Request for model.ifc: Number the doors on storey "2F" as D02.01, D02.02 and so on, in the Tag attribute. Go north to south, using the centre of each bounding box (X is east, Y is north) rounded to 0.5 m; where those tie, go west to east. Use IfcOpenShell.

First a look at what the model holds.

```python
import ifcopenshell
import ifcopenshell.util.element
import ifcopenshell.util.placement

model = ifcopenshell.open("model.ifc")
print(model.schema)
storey = next(s for s in model.by_type("IfcBuildingStorey") if s.Name == "2F")
doors = [e for e in ifcopenshell.util.element.get_decomposition(storey) if e.is_a("IfcDoor")]
for e in sorted(doors, key=lambda e: e.id()):
    origin = ifcopenshell.util.placement.get_local_placement(e.ObjectPlacement)[:3, 3]
    print(e.id(), e.Tag, e.Name, origin.round(2) + 0.0, sep=" | ")
```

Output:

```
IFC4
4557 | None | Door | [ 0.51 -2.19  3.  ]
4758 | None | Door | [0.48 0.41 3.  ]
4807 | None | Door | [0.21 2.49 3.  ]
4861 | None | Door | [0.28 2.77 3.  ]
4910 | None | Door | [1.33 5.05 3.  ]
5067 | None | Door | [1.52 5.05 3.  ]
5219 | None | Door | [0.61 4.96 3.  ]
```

```python
import ifcopenshell
import ifcopenshell.geom
import ifcopenshell.util.element
import ifcopenshell.util.shape

model = ifcopenshell.open("model.ifc")
settings = ifcopenshell.geom.settings()
settings.set("use-world-coords", True)


def centre(element):
    shape = ifcopenshell.geom.create_shape(settings, element)
    return ifcopenshell.util.shape.get_bbox_centroid(shape.geometry)


storey = next(s for s in model.by_type("IfcBuildingStorey") if s.Name == "2F")
doors = [e for e in ifcopenshell.util.element.get_decomposition(storey) if e.is_a("IfcDoor")]

# Insertion points can sit at a corner or the storey origin, so sort by the geometry (in metres).
centres = {e: centre(e) for e in doors}
doors.sort(key=lambda e: (-round(centres[e][1] / 0.5), centres[e][0]))

for i, e in enumerate(doors, start=1):
    number = f"D02.{i:02d}"
    e.Tag = number
    print(e.id(), number)

model.write("model-out.ifc")
```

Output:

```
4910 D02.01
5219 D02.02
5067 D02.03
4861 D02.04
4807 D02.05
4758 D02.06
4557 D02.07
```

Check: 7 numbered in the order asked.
